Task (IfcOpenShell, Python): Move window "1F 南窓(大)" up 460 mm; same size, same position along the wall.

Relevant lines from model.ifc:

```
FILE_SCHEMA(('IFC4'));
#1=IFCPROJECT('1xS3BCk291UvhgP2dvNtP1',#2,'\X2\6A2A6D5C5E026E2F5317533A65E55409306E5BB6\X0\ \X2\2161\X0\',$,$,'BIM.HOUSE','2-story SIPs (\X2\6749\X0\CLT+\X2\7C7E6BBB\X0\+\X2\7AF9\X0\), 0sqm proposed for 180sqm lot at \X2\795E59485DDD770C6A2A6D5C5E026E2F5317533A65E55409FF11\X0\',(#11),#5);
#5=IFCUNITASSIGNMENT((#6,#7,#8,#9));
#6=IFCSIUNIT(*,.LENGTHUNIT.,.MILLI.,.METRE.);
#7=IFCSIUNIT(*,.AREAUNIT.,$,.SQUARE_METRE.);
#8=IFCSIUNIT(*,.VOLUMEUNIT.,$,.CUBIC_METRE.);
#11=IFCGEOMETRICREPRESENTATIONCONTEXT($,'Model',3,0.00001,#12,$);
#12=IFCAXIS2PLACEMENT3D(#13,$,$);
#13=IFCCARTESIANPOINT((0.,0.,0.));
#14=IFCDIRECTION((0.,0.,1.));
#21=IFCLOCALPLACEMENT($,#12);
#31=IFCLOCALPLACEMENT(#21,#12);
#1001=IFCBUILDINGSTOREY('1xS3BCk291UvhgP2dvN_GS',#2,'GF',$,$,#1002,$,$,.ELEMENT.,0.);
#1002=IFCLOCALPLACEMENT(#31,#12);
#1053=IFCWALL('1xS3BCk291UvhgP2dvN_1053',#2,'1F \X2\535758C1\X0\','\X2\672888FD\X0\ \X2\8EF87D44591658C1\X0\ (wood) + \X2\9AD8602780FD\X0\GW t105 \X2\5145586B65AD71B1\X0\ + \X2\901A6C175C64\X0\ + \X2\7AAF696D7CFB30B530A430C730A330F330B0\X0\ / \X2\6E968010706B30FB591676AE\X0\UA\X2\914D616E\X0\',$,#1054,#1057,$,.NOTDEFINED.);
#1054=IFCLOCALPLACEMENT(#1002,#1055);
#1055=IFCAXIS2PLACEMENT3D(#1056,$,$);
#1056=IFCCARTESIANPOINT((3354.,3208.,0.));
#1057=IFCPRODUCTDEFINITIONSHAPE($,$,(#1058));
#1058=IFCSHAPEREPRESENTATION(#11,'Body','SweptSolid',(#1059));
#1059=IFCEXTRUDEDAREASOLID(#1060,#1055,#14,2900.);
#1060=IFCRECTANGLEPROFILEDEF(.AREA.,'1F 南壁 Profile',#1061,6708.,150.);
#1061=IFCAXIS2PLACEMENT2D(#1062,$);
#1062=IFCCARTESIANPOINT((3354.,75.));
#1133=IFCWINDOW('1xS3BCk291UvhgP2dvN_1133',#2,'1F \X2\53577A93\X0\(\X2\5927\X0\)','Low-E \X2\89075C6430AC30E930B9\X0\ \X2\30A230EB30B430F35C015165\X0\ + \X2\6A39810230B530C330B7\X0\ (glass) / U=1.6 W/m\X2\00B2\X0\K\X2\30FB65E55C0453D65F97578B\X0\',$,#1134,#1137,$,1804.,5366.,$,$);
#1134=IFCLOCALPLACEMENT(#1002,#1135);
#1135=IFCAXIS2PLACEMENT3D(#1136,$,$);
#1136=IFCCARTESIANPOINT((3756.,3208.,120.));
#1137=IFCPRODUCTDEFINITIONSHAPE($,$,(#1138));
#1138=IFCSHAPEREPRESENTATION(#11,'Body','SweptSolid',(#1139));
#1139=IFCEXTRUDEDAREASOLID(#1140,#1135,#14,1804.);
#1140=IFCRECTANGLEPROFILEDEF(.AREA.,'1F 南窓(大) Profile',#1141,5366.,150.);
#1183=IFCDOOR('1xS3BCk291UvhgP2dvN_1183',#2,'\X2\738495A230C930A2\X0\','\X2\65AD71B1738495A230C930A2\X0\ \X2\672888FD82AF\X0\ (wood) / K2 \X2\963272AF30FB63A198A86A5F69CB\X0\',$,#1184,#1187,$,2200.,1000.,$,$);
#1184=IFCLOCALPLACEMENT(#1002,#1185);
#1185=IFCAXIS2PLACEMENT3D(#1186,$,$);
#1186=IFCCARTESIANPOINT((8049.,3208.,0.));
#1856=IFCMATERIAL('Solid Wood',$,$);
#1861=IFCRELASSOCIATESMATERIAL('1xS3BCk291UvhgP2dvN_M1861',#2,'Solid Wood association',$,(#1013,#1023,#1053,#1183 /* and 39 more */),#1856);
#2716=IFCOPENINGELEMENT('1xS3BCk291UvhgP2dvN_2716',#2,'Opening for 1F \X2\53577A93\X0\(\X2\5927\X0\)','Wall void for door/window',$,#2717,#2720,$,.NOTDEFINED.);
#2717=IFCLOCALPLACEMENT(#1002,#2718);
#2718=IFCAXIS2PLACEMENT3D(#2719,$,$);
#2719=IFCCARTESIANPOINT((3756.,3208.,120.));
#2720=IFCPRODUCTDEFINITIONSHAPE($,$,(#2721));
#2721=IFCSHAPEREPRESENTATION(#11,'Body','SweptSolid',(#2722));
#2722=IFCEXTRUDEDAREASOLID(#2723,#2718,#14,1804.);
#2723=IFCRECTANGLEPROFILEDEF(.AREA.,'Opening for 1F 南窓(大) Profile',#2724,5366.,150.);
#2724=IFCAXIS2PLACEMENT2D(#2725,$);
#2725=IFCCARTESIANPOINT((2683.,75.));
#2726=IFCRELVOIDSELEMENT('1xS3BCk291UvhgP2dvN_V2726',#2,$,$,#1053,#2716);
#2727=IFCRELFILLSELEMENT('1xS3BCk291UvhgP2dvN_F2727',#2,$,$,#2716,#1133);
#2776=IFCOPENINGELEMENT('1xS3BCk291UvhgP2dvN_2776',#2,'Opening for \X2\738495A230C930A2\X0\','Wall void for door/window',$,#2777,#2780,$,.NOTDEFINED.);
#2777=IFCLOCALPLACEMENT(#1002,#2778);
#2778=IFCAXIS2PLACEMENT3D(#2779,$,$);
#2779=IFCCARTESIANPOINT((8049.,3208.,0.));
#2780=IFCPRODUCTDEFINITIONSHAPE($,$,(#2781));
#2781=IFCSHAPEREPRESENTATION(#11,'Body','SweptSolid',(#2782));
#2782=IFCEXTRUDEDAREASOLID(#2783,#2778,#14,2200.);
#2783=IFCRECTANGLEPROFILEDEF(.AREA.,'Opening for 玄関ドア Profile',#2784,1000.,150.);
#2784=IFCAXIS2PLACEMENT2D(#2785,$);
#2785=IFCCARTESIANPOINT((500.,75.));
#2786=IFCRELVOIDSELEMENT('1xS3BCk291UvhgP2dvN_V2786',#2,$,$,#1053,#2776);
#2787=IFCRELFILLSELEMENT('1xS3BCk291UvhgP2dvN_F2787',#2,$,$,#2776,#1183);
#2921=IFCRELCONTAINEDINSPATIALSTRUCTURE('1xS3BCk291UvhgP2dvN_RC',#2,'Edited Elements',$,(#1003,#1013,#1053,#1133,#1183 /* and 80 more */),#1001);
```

```python
import numpy as np
import ifcopenshell
import ifcopenshell.api.geometry
import ifcopenshell.util.placement
import ifcopenshell.util.unit

model = ifcopenshell.open("model.ifc")
unit_scale = ifcopenshell.util.unit.calculate_unit_scale(model)

window = model.by_guid("1xS3BCk291UvhgP2dvN_1133")
opening = window.FillsVoids[0].RelatingOpeningElement
dz = 0.46 / unit_scale

shift = np.array([0.0, 0.0, dz])
# The window is not placed relative to its opening, so move both.
for product in (opening, window):
    matrix = ifcopenshell.util.placement.get_local_placement(product.ObjectPlacement)
    matrix[:3, 3] += shift
    ifcopenshell.api.geometry.edit_object_placement(model, product=product, matrix=matrix, is_si=False)

print(f"moved by {dz * unit_scale:+.3f} m")

model.write("model_edited.ifc")
```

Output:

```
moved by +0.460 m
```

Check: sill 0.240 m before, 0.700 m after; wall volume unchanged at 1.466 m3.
